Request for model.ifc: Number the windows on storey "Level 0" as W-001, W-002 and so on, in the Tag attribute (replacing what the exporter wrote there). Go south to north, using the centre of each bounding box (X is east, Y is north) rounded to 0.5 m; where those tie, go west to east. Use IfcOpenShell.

First a look at what the model holds.

```python
import ifcopenshell
import ifcopenshell.util.element
import ifcopenshell.util.placement

model = ifcopenshell.open("model.ifc")
print(model.schema)
storey = next(s for s in model.by_type("IfcBuildingStorey") if s.Name == "Level 0")
windows = [e for e in ifcopenshell.util.element.get_decomposition(storey) if e.is_a("IfcWindow")]
for e in sorted(windows, key=lambda e: e.id()):
    origin = ifcopenshell.util.placement.get_local_placement(e.ObjectPlacement)[:3, 3]
    print(e.id(), e.Tag, e.Name, origin.round(2) + 0.0, sep=" | ")
```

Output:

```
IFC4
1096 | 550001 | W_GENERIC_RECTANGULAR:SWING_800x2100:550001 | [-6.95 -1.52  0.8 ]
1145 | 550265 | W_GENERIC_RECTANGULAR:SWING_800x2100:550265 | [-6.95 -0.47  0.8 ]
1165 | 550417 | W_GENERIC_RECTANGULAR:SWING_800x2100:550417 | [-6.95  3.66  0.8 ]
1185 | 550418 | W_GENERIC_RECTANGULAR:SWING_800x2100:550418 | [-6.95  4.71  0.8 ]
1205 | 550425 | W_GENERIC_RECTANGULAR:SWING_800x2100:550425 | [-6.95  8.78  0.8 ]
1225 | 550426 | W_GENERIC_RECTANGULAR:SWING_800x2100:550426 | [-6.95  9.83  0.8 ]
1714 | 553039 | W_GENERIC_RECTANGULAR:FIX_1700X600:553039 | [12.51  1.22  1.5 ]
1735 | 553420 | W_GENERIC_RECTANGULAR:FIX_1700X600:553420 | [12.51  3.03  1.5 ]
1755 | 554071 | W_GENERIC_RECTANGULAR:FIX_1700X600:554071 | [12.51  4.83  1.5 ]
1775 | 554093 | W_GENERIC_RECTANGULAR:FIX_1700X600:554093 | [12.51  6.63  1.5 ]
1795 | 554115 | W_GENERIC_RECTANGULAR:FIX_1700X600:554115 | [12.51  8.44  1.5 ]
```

```python
import ifcopenshell
import ifcopenshell.geom
import ifcopenshell.util.element
import ifcopenshell.util.shape

model = ifcopenshell.open("model.ifc")
settings = ifcopenshell.geom.settings()
settings.set("use-world-coords", True)


def centre(element):
    shape = ifcopenshell.geom.create_shape(settings, element)
    return ifcopenshell.util.shape.get_bbox_centroid(shape.geometry)


storey = next(s for s in model.by_type("IfcBuildingStorey") if s.Name == "Level 0")
windows = [e for e in ifcopenshell.util.element.get_decomposition(storey) if e.is_a("IfcWindow")]

# Insertion points can sit at a corner or the storey origin, so sort by the geometry (in metres).
centres = {e: centre(e) for e in windows}
windows.sort(key=lambda e: (round(centres[e][1] / 0.5), centres[e][0]))

for i, e in enumerate(windows, start=1):
    number = f"W-0{i:02d}"
    e.Tag = number
    print(e.id(), number)

model.write("model_v2.ifc")
```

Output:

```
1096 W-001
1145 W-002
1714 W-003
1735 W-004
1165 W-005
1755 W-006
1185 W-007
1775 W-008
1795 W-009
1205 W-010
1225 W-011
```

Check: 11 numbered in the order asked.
